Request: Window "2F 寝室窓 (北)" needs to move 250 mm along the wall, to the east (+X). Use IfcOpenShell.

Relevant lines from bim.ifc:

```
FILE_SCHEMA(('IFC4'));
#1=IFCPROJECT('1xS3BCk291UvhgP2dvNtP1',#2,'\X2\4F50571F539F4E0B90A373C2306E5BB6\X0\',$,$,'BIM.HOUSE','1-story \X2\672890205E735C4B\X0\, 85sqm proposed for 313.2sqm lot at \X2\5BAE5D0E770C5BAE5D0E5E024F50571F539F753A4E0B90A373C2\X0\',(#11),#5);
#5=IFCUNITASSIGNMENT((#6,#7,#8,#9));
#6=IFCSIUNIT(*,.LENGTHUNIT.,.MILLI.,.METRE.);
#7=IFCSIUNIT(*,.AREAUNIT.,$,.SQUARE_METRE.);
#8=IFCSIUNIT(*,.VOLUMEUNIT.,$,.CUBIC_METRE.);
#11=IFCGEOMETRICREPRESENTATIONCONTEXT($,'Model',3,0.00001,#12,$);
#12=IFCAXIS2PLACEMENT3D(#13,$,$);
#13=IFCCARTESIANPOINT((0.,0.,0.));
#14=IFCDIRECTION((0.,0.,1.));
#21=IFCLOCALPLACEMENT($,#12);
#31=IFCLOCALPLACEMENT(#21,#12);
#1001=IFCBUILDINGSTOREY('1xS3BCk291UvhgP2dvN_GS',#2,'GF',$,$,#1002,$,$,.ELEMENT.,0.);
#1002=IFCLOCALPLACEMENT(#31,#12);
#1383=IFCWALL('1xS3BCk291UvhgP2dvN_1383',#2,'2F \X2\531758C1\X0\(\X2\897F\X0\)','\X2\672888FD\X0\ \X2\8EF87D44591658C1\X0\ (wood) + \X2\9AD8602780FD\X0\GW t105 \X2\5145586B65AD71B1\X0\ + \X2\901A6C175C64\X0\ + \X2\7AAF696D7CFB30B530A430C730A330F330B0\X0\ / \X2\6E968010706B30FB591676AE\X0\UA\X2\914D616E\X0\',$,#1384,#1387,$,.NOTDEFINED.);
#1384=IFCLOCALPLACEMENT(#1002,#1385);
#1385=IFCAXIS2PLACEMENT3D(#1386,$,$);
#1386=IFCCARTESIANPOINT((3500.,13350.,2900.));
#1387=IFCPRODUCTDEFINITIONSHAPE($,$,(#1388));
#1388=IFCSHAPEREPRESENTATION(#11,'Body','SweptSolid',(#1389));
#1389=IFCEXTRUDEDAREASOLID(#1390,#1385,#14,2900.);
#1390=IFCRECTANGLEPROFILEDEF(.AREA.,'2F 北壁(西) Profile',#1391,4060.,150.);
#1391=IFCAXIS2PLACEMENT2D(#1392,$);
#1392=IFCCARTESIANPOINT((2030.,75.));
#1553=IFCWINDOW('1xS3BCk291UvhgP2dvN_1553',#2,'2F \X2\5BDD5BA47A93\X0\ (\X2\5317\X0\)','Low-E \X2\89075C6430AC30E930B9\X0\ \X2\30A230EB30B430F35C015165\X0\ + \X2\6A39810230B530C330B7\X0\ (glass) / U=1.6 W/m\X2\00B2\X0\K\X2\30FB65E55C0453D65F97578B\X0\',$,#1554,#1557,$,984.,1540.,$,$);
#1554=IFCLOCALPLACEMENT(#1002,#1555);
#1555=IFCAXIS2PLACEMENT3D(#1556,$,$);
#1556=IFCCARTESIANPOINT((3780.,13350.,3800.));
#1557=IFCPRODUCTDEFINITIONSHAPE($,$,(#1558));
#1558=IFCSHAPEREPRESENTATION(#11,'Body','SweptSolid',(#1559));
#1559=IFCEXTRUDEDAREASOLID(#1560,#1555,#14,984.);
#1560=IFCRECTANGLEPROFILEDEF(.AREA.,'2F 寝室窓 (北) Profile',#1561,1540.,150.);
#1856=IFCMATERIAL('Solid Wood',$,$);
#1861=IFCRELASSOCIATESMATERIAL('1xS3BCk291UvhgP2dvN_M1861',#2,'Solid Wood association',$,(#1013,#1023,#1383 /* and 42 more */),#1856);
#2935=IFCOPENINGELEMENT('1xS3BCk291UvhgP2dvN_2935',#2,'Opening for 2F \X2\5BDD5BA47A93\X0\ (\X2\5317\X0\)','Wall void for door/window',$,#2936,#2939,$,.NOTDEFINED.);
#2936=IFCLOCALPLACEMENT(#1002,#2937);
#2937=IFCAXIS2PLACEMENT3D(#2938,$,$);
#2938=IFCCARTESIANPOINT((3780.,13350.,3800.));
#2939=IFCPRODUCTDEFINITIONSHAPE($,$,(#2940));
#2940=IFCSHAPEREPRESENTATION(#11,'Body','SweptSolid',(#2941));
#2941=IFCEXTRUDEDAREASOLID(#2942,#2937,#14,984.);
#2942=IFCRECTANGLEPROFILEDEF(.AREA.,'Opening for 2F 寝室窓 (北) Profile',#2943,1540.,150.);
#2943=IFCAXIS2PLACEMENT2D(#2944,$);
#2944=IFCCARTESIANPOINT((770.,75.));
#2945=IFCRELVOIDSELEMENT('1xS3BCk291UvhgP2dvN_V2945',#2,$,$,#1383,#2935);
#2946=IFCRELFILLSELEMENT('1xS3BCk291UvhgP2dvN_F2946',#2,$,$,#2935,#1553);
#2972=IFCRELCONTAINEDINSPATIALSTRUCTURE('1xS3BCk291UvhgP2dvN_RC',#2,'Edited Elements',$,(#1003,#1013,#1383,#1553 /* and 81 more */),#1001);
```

```python
import ifcopenshell
import ifcopenshell.api.geometry
import ifcopenshell.util.placement

model = ifcopenshell.open("bim.ifc")

window = model.by_id(1553)
opening = window.FillsVoids[0].RelatingOpeningElement
wall = opening.VoidsElements[0].RelatingBuildingElement

wall_matrix = ifcopenshell.util.placement.get_local_placement(wall.ObjectPlacement)
shift = wall_matrix[:3, 0] * 250.0
before = ifcopenshell.util.placement.get_local_placement(window.ObjectPlacement)[:3, 3].copy()

# The window is not placed relative to its opening, so move both.
for product in (opening, window):
    matrix = ifcopenshell.util.placement.get_local_placement(product.ObjectPlacement)
    matrix[:3, 3] += shift
    ifcopenshell.api.geometry.edit_object_placement(model, product=product, matrix=matrix, is_si=False)

after = ifcopenshell.util.placement.get_local_placement(window.ObjectPlacement)[:3, 3]
print("window moved by", (after - before).round(3) + 0.0)

model.write("bim_edited.ifc")
```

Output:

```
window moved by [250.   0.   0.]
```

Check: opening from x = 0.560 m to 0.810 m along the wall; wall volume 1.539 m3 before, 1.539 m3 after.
